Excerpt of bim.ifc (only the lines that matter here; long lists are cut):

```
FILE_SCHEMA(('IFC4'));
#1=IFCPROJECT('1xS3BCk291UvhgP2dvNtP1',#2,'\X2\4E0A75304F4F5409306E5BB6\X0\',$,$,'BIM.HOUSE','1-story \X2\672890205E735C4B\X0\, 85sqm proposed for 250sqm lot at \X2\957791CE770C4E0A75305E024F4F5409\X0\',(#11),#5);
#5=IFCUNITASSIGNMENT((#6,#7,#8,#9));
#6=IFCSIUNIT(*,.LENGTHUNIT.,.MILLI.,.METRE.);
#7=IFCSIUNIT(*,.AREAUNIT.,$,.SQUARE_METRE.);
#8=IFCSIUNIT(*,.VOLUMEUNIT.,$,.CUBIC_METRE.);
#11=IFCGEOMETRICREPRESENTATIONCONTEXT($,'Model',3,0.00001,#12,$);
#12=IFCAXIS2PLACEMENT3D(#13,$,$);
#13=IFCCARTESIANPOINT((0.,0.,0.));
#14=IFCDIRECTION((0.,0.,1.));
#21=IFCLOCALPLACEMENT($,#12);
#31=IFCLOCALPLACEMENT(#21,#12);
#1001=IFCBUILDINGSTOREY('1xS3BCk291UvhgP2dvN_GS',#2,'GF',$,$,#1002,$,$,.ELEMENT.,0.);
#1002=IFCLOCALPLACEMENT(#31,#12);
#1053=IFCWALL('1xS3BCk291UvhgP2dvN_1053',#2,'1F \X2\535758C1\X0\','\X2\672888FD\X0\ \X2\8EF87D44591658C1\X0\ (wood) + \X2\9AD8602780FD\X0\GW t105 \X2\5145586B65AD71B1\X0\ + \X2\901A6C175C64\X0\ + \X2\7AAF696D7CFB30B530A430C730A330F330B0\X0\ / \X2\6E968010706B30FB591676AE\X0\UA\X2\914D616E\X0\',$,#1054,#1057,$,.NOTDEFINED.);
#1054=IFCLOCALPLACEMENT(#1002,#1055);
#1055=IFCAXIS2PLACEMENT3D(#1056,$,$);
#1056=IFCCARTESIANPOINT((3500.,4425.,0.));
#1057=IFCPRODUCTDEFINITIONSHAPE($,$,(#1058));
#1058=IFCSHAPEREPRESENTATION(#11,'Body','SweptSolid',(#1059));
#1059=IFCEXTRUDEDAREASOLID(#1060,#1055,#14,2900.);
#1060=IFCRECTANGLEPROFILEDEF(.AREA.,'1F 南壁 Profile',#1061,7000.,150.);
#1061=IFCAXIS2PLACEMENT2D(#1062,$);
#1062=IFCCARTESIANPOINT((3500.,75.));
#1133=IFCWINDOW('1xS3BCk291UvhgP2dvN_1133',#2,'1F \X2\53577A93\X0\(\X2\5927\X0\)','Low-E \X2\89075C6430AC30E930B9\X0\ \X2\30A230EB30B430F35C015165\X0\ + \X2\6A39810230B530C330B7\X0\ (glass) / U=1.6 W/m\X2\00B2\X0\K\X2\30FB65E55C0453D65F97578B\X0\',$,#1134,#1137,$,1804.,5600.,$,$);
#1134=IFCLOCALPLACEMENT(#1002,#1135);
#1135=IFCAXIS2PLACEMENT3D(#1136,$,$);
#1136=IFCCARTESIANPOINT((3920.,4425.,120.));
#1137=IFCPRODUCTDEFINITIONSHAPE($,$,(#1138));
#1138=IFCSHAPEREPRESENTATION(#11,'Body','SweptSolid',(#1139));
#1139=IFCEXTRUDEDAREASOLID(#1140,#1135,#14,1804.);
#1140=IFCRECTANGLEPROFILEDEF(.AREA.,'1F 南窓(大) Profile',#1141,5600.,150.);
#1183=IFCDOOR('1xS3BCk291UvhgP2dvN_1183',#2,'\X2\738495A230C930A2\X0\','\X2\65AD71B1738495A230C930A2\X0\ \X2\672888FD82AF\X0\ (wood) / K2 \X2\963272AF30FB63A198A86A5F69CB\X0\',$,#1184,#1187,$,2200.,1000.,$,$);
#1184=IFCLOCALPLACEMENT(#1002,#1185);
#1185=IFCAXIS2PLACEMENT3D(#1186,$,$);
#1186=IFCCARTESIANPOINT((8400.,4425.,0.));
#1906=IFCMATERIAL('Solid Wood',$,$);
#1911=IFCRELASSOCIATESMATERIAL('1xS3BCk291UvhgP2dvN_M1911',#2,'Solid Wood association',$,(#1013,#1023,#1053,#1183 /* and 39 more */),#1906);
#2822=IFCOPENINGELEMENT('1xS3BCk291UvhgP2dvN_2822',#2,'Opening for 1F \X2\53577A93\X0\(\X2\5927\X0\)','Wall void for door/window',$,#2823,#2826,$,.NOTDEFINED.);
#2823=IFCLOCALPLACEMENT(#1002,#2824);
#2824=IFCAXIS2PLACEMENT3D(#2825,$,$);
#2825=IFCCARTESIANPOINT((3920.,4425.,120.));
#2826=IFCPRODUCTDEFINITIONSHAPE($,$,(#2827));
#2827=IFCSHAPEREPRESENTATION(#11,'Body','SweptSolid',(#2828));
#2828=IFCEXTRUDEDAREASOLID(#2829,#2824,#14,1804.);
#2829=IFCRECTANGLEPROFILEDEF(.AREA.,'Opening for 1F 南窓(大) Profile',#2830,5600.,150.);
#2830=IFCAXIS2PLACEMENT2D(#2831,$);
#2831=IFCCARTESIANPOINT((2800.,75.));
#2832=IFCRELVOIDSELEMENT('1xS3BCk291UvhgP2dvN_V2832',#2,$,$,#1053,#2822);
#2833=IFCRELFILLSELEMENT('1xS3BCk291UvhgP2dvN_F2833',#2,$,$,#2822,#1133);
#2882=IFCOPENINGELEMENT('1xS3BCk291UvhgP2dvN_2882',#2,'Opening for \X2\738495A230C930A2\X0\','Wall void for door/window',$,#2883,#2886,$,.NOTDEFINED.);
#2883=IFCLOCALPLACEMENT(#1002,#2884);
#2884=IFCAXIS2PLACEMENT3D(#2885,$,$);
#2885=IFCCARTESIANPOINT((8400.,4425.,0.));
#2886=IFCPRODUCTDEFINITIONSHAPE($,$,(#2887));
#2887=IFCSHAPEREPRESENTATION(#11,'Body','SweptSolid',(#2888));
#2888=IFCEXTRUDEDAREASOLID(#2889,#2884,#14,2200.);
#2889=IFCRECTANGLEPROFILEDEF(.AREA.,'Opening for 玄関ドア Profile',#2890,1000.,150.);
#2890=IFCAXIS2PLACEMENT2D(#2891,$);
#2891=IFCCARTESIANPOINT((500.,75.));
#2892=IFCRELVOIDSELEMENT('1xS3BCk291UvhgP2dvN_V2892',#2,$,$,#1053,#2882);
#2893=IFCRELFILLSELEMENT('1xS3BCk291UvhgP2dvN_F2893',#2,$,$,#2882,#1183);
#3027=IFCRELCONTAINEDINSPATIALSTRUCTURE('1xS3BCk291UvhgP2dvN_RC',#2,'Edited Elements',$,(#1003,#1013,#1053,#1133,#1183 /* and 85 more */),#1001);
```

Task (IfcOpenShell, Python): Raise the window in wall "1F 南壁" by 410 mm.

```python
import numpy as np
import ifcopenshell
import ifcopenshell.api.geometry
import ifcopenshell.util.placement
import ifcopenshell.util.unit

model = ifcopenshell.open("bim.ifc")
unit_scale = ifcopenshell.util.unit.calculate_unit_scale(model)

window = model.by_guid("1xS3BCk291UvhgP2dvN_1133")
opening = window.FillsVoids[0].RelatingOpeningElement
dz = 0.41 / unit_scale

shift = np.array([0.0, 0.0, dz])
# The window is not placed relative to its opening, so move both.
for product in (opening, window):
    matrix = ifcopenshell.util.placement.get_local_placement(product.ObjectPlacement)
    matrix[:3, 3] += shift
    ifcopenshell.api.geometry.edit_object_placement(model, product=product, matrix=matrix, is_si=False)

print(f"moved by {dz * unit_scale:+.3f} m")

model.write("bim_edited.ifc")
```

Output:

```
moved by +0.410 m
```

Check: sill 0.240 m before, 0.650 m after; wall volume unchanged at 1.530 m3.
